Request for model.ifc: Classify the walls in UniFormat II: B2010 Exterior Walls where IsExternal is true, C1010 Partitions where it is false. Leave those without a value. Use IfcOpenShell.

First a look at what the model holds.

```python
import ifcopenshell
import ifcopenshell.util.element

model = ifcopenshell.open("model.ifc")
print(model.schema)
print("classifications:", [c.Name for c in model.by_type("IfcClassification")])
values = [ifcopenshell.util.element.get_pset(e, "Pset_WallCommon", "IsExternal") for e in model.by_type("IfcWall")]
for value in (True, False, None):
    print("IsExternal", value, values.count(value))
```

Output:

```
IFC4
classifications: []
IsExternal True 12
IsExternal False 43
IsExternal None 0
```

```python
import ifcopenshell
import ifcopenshell.api.classification
import ifcopenshell.util.element

model = ifcopenshell.open("model.ifc")

system = ifcopenshell.api.classification.add_classification(model, classification="UniFormat II")

walls = model.by_type("IfcWall")
external = {e: ifcopenshell.util.element.get_pset(e, "Pset_WallCommon", "IsExternal") for e in walls}
for flag, code, name in ((True, "B2010", "Exterior Walls"), (False, "C1010", "Partitions")):
    products = [e for e in walls if external[e] is flag]
    ifcopenshell.api.classification.add_reference(
        model, products=products, classification=system, identification=code, name=name
    )
    print(code, len(products))

model.write("model_updated.ifc")
```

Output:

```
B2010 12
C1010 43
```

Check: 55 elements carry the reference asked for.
